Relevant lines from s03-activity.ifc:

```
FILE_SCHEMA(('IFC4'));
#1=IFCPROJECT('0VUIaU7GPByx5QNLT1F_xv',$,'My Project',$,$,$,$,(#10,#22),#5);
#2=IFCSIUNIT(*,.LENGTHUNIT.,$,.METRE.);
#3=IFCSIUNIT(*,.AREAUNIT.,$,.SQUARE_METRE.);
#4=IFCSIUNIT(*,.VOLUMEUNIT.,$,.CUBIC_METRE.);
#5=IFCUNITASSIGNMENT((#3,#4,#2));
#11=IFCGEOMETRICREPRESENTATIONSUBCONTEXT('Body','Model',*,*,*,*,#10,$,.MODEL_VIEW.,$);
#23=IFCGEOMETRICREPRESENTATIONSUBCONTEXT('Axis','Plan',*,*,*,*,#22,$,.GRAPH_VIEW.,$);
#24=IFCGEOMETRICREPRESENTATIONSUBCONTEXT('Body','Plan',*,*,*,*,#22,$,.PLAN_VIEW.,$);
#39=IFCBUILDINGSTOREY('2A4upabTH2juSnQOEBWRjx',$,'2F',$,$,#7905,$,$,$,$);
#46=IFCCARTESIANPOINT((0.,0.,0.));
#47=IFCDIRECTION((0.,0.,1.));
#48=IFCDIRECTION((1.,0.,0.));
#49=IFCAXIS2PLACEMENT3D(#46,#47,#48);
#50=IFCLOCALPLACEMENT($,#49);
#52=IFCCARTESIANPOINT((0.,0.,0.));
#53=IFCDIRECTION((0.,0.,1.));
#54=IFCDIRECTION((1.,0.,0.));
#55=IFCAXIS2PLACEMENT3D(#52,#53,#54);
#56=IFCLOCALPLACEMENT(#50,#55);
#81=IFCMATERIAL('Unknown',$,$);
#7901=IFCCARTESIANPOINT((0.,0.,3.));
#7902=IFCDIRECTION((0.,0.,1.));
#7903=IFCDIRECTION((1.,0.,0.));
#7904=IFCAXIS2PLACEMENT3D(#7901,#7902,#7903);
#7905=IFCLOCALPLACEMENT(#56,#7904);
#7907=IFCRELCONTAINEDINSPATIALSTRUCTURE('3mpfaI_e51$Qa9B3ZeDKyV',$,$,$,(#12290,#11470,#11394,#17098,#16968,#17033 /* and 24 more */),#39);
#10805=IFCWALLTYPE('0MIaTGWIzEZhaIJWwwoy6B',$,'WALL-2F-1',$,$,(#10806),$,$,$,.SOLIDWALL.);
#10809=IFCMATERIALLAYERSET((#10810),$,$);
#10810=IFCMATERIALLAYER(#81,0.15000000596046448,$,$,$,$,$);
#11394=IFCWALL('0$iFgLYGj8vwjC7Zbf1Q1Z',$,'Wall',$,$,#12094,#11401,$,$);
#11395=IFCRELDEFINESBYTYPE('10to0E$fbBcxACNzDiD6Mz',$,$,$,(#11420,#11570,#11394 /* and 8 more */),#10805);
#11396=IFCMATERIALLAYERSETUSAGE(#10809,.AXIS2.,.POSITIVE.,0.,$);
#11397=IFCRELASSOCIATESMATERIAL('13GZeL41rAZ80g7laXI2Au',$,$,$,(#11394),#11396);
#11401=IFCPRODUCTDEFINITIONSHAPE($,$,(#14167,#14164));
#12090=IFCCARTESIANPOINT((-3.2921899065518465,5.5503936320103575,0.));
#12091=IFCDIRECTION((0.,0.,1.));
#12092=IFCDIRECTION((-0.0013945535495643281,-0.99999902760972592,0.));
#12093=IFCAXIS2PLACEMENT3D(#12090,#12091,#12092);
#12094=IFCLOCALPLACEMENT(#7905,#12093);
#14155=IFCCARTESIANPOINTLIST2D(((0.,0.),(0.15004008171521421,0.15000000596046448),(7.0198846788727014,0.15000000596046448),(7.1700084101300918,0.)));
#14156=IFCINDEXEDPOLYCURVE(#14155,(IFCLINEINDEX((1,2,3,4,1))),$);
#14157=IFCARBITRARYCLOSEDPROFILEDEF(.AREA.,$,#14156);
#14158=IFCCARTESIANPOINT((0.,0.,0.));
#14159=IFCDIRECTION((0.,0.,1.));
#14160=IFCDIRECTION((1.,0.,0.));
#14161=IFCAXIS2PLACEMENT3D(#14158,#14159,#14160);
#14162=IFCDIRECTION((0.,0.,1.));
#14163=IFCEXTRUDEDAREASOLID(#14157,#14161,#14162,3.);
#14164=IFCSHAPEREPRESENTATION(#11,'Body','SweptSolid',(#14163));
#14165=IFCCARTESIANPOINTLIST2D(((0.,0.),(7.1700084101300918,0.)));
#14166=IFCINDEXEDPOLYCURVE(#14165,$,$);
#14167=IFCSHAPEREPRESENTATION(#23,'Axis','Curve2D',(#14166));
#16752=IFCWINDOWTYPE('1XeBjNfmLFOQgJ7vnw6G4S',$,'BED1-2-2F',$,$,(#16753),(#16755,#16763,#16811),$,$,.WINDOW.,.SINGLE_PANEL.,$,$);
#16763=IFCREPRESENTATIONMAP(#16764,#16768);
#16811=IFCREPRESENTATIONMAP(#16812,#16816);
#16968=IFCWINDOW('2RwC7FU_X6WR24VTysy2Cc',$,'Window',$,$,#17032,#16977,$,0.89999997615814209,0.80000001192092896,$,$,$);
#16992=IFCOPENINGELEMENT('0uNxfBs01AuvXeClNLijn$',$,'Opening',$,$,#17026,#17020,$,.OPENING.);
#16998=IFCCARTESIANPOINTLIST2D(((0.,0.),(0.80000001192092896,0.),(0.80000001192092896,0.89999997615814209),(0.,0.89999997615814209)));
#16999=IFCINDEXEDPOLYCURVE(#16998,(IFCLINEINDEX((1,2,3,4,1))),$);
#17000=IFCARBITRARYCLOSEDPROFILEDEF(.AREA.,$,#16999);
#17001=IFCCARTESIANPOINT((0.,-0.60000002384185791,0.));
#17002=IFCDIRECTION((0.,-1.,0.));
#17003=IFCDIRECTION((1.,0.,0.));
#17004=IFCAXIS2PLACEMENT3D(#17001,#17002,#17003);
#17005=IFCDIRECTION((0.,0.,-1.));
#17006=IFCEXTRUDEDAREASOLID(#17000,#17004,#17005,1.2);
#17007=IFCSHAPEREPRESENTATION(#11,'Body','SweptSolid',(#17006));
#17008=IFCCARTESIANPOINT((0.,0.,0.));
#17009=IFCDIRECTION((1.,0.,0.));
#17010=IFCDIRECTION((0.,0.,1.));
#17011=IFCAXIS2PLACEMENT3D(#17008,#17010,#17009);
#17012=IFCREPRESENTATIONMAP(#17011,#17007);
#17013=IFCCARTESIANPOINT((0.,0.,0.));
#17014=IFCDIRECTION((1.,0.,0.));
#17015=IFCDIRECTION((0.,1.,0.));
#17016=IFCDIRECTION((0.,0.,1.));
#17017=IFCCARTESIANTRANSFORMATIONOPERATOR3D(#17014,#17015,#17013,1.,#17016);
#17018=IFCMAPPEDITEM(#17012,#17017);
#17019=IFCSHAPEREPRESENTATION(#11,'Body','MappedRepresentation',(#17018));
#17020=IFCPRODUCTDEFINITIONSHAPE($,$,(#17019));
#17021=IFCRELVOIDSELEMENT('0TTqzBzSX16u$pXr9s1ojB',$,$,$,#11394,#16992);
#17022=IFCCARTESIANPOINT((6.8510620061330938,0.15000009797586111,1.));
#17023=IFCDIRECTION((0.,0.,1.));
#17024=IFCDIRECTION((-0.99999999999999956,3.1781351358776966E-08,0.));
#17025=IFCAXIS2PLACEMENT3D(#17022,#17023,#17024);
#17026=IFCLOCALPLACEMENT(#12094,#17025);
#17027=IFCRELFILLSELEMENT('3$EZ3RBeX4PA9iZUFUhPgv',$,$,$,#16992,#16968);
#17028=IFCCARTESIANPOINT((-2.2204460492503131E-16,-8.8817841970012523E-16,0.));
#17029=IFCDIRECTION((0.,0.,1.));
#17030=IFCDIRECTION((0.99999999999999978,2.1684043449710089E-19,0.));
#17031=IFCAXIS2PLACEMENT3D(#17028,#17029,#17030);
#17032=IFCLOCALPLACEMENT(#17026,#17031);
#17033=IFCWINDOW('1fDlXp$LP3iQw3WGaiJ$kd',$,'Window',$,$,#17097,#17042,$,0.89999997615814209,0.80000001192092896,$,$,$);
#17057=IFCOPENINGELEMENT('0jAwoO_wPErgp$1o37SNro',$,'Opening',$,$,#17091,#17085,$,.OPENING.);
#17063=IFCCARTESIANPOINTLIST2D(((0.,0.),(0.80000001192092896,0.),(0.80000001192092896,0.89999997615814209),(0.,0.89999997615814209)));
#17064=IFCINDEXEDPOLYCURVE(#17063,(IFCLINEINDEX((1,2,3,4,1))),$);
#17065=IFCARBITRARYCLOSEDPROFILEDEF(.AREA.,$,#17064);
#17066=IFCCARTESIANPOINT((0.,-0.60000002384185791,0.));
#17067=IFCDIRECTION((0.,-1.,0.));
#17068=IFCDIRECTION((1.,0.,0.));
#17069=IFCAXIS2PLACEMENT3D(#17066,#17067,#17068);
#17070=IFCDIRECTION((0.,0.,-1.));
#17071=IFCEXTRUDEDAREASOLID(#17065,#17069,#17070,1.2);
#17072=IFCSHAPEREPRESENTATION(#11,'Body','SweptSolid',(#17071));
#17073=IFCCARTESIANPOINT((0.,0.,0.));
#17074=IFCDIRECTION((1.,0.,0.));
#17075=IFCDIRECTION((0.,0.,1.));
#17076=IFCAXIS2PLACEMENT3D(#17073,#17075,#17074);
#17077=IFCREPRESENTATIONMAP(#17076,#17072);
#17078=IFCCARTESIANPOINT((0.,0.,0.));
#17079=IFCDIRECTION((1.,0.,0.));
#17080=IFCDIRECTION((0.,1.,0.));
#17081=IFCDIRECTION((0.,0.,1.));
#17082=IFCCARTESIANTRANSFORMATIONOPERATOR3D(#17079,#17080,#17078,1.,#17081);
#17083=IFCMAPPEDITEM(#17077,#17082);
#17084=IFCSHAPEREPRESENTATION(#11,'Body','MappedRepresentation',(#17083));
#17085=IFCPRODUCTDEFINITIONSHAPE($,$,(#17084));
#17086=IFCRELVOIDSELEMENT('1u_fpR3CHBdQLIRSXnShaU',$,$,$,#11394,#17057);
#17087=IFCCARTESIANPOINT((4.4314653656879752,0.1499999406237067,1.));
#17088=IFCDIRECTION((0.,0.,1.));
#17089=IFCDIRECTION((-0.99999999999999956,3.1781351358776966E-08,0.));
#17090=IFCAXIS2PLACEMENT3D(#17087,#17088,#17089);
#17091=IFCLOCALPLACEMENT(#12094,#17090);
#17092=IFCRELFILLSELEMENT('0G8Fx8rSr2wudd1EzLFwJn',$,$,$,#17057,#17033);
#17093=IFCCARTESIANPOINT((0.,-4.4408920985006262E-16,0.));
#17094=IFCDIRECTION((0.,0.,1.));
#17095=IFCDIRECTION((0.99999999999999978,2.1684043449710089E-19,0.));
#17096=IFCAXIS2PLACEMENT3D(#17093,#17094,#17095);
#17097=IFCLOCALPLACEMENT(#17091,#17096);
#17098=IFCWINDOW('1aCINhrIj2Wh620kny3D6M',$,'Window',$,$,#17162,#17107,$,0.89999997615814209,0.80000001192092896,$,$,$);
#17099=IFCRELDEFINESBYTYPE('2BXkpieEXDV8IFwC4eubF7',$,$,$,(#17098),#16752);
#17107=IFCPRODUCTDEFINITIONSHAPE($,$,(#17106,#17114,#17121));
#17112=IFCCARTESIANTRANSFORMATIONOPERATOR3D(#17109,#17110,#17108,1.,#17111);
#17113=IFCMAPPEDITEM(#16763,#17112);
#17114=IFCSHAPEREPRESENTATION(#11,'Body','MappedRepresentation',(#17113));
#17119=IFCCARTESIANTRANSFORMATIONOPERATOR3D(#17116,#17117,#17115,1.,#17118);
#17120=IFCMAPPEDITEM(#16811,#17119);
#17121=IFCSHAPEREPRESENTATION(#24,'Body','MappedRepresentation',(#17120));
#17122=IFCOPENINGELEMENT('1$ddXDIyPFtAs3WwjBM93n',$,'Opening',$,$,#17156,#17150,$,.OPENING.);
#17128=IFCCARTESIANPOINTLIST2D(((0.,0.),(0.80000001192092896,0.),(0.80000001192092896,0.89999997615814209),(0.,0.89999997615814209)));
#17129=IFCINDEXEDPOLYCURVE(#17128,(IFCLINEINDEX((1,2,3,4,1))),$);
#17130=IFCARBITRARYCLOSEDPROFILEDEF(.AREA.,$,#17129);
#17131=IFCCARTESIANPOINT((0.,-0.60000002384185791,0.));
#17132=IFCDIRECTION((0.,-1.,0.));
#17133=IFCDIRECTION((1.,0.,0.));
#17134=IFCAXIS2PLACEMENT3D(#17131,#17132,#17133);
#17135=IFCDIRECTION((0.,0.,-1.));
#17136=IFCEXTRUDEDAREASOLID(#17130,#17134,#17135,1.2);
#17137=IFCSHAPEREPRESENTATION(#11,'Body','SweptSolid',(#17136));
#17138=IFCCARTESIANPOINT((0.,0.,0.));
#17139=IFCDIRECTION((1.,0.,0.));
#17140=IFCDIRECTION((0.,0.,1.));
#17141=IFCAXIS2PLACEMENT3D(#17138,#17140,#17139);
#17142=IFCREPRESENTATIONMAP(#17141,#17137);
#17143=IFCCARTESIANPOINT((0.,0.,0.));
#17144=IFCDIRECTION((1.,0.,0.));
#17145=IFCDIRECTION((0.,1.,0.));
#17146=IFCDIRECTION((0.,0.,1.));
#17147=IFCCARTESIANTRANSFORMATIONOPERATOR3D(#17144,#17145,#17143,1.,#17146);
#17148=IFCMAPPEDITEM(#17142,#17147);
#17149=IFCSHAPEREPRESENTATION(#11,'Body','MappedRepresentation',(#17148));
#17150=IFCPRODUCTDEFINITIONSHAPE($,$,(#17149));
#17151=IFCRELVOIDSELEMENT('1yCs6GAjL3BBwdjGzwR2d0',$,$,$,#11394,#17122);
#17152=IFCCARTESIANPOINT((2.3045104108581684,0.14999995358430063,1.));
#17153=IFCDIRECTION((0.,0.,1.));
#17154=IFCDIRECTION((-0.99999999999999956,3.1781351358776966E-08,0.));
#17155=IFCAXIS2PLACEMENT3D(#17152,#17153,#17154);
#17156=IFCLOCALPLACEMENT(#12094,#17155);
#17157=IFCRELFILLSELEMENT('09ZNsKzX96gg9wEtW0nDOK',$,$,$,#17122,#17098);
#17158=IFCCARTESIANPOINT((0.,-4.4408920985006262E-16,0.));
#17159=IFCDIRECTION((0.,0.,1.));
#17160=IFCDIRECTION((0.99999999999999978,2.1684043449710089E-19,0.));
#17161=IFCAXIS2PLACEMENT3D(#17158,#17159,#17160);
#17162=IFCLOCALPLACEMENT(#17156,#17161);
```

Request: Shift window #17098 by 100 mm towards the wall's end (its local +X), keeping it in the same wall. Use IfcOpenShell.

```python
import ifcopenshell
import ifcopenshell.api.geometry
import ifcopenshell.util.placement
import ifcopenshell.util.unit

model = ifcopenshell.open("s03-activity.ifc")
unit_scale = ifcopenshell.util.unit.calculate_unit_scale(model)

window = model.by_guid("1aCINhrIj2Wh620kny3D6M")
opening = window.FillsVoids[0].RelatingOpeningElement
wall = opening.VoidsElements[0].RelatingBuildingElement

wall_matrix = ifcopenshell.util.placement.get_local_placement(wall.ObjectPlacement)
shift = wall_matrix[:3, 0] * 0.1 / unit_scale
before = ifcopenshell.util.placement.get_local_placement(window.ObjectPlacement)[:3, 3].copy()

# The window is placed relative to its opening, so it follows when the opening moves.
matrix = ifcopenshell.util.placement.get_local_placement(opening.ObjectPlacement)
matrix[:3, 3] += shift
ifcopenshell.api.geometry.edit_object_placement(
    model, product=opening, matrix=matrix, is_si=False, should_transform_children=True
)

after = ifcopenshell.util.placement.get_local_placement(window.ObjectPlacement)[:3, 3]
print("window moved by", (after - before).round(3) + 0.0)

model.write("s03-activity_v2.ifc")
```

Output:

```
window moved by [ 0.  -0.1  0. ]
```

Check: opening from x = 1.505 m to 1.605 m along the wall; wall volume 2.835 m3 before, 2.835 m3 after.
